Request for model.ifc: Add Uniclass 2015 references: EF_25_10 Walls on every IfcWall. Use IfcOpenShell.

First a look at what the model holds.

```python
import ifcopenshell

model = ifcopenshell.open("model.ifc")
print(model.schema)
print("classifications:", [c.Name for c in model.by_type("IfcClassification")])
for ifc_class in ("IfcDoor", "IfcRoof", "IfcStair", "IfcWall", "IfcWindow"):
    print(ifc_class, len(model.by_type(ifc_class)))
```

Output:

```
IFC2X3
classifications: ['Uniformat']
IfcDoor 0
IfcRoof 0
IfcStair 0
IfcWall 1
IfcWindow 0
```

```python
import ifcopenshell
import ifcopenshell.api.classification

model = ifcopenshell.open("model.ifc")

# IFC2X3 requires Source and Edition and has no link from the project to the system.
system = model.create_entity("IfcClassification", Source="NBS", Edition="2015", Name="Uniclass 2015")

codes = {
    "IfcWall": ("EF_25_10", "Walls"),
}
for ifc_class, (code, name) in codes.items():
    products = model.by_type(ifc_class)
    ifcopenshell.api.classification.add_reference(
        model, products=products, classification=system, identification=code, name=name
    )
    print(code, len(products))

model.write("model_v2.ifc")
```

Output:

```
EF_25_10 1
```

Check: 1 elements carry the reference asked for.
